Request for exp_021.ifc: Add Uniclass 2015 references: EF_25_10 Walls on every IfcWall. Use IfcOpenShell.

First a look at what the model holds.

```python
import ifcopenshell

model = ifcopenshell.open("exp_021.ifc")
print(model.schema)
print("classifications:", [c.Name for c in model.by_type("IfcClassification")])
for ifc_class in ("IfcDoor", "IfcRoof", "IfcStair", "IfcWall", "IfcWindow"):
    print(ifc_class, len(model.by_type(ifc_class)))
```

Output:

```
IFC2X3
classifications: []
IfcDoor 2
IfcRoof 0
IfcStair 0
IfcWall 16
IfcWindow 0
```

```python
import ifcopenshell
import ifcopenshell.api.classification

model = ifcopenshell.open("exp_021.ifc")

# IFC2X3 requires Source and Edition and has no link from the project to the system.
system = model.create_entity("IfcClassification", Source="NBS", Edition="2015", Name="Uniclass 2015")

codes = {
    "IfcWall": ("EF_25_10", "Walls"),
}
for ifc_class, (code, name) in codes.items():
    products = model.by_type(ifc_class)
    ifcopenshell.api.classification.add_reference(
        model, products=products, classification=system, identification=code, name=name
    )
    print(code, len(products))

model.write("exp_021_v2.ifc")
```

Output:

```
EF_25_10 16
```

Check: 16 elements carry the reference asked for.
